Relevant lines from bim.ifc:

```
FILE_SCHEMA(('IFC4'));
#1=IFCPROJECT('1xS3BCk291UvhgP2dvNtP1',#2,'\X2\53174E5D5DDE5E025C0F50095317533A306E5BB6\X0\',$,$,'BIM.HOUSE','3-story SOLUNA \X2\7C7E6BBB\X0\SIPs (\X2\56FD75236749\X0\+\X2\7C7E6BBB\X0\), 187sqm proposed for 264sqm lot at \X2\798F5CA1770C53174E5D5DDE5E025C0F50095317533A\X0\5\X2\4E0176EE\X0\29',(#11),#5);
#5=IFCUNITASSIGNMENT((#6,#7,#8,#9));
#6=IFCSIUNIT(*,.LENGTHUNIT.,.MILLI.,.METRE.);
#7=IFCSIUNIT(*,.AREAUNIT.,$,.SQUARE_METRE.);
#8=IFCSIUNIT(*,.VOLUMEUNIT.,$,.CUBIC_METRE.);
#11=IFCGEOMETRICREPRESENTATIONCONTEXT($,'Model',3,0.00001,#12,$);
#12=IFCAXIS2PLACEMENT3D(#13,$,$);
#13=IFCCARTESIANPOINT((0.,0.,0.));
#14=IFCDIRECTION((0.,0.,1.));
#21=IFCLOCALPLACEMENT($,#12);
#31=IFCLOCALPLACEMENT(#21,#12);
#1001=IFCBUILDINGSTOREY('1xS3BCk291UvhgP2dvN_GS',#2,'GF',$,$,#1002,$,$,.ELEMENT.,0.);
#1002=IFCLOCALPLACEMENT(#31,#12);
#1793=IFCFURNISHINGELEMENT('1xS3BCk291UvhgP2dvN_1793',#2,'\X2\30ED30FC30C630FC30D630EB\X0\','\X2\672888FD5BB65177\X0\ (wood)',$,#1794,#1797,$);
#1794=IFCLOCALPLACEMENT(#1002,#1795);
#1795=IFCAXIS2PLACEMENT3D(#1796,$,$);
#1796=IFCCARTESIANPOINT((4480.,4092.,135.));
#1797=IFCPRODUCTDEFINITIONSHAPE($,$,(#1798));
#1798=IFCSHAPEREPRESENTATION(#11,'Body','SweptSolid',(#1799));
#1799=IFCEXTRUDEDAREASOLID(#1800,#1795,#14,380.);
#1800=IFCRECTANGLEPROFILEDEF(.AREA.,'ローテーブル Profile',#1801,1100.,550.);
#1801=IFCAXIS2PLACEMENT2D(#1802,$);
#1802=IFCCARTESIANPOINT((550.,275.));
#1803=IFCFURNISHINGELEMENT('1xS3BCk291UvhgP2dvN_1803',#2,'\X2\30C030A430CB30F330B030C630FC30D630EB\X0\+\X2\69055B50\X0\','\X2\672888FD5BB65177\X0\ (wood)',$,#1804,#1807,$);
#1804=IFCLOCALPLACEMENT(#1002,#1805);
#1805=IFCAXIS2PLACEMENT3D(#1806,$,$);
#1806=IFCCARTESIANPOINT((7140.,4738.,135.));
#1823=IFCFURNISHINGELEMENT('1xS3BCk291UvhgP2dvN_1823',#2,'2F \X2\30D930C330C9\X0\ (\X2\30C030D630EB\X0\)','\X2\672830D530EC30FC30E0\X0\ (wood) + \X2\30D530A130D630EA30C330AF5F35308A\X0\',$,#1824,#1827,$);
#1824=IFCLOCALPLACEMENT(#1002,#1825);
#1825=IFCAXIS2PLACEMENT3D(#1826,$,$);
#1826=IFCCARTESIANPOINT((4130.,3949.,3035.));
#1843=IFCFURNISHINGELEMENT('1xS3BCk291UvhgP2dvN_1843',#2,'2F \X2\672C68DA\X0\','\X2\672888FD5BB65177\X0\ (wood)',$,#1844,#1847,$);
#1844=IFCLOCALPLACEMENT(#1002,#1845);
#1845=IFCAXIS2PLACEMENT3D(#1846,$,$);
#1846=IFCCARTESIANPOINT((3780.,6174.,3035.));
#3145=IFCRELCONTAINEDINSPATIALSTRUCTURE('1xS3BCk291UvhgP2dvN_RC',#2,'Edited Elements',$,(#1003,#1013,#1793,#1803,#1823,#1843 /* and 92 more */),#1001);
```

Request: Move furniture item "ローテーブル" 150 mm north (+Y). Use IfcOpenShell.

```python
import ifcopenshell
import ifcopenshell.api.geometry
import ifcopenshell.util.placement
import ifcopenshell.util.unit

model = ifcopenshell.open("bim.ifc")
unit_scale = ifcopenshell.util.unit.calculate_unit_scale(model)

item = model.by_guid("1xS3BCk291UvhgP2dvN_1793")
matrix = ifcopenshell.util.placement.get_local_placement(item.ObjectPlacement)
matrix[1, 3] += 0.15 / unit_scale
ifcopenshell.api.geometry.edit_object_placement(model, product=item, matrix=matrix, is_si=False)

print(ifcopenshell.util.placement.get_local_placement(item.ObjectPlacement).round(3) + 0.0)

model.write("bim_edited.ifc")
```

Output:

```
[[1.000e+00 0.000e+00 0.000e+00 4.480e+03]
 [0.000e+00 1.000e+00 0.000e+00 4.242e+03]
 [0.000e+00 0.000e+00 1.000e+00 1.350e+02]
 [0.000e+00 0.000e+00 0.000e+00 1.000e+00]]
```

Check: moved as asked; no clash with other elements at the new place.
